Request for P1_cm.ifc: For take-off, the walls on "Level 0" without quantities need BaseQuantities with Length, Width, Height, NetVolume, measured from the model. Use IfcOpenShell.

First a look at what the model holds.

```python
import ifcopenshell
import ifcopenshell.util.element
import ifcopenshell.util.unit

model = ifcopenshell.open("P1_cm.ifc")
print(model.schema)
for unit_type in ("LENGTHUNIT", "AREAUNIT", "VOLUMEUNIT"):
    print(unit_type, ifcopenshell.util.unit.calculate_unit_scale(model, unit_type))
storey = next(s for s in model.by_type("IfcBuildingStorey") if s.Name == "Level 0")
walls = [e for e in ifcopenshell.util.element.get_decomposition(storey) if e.is_a("IfcWall")]
for e in sorted(walls, key=lambda e: e.id()):
    print(e.id(), e.is_a(), e.Name, list(ifcopenshell.util.element.get_psets(e, qtos_only=True)), sep=" | ")
```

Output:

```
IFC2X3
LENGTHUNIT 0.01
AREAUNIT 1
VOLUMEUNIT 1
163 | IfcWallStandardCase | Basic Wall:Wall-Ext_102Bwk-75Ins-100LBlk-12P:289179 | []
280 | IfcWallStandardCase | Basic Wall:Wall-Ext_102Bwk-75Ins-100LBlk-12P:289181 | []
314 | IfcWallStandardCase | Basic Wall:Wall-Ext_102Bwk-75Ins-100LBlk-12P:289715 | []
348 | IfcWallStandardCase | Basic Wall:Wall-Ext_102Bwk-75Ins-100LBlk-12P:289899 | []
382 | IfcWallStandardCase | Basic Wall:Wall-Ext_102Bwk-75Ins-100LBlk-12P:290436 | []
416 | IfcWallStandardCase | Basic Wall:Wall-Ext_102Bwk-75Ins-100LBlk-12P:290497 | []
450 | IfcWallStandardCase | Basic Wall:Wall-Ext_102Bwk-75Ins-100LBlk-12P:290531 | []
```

```python
import ifcopenshell
import ifcopenshell.api.pset
import ifcopenshell.geom
import ifcopenshell.util.element
import ifcopenshell.util.shape
import ifcopenshell.util.unit

model = ifcopenshell.open("P1_cm.ifc")
unit_scale = ifcopenshell.util.unit.calculate_unit_scale(model)
volume_scale = ifcopenshell.util.unit.calculate_unit_scale(model, "VOLUMEUNIT")
settings = ifcopenshell.geom.settings()

storey = next(s for s in model.by_type("IfcBuildingStorey") if s.Name == "Level 0")
walls = [e for e in ifcopenshell.util.element.get_decomposition(storey) if e.is_a("IfcWall")]

for e in sorted(walls, key=lambda e: e.id()):
    if ifcopenshell.util.element.get_psets(e, qtos_only=True, should_inherit=False):
        continue
    # Geometry comes back in metres, in the element's own axes.
    shape = ifcopenshell.geom.create_shape(settings, e)
    values = {
        "Length": ifcopenshell.util.shape.get_x(shape.geometry) / unit_scale,
        "Width": ifcopenshell.util.shape.get_y(shape.geometry) / unit_scale,
        "Height": ifcopenshell.util.shape.get_z(shape.geometry) / unit_scale,
        "NetVolume": ifcopenshell.util.shape.get_volume(shape.geometry) / volume_scale,
    }
    qto = ifcopenshell.api.pset.add_qto(model, product=e, name="BaseQuantities")
    ifcopenshell.api.pset.edit_qto(model, qto=qto, properties=values)
    print(e.id(), {k: round(v, 3) for k, v in values.items()})

model.write("P1_cm_updated.ifc")
```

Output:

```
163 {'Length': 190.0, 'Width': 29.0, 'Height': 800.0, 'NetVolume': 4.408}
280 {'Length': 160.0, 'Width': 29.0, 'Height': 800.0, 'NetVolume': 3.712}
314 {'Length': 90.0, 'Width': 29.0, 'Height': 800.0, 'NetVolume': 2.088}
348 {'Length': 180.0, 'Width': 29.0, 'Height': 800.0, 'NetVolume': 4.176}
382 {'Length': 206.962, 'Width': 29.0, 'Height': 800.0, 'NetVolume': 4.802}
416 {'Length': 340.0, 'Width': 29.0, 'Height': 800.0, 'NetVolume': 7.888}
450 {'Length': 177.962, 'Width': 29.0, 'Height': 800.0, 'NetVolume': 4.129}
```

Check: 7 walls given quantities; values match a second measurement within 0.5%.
